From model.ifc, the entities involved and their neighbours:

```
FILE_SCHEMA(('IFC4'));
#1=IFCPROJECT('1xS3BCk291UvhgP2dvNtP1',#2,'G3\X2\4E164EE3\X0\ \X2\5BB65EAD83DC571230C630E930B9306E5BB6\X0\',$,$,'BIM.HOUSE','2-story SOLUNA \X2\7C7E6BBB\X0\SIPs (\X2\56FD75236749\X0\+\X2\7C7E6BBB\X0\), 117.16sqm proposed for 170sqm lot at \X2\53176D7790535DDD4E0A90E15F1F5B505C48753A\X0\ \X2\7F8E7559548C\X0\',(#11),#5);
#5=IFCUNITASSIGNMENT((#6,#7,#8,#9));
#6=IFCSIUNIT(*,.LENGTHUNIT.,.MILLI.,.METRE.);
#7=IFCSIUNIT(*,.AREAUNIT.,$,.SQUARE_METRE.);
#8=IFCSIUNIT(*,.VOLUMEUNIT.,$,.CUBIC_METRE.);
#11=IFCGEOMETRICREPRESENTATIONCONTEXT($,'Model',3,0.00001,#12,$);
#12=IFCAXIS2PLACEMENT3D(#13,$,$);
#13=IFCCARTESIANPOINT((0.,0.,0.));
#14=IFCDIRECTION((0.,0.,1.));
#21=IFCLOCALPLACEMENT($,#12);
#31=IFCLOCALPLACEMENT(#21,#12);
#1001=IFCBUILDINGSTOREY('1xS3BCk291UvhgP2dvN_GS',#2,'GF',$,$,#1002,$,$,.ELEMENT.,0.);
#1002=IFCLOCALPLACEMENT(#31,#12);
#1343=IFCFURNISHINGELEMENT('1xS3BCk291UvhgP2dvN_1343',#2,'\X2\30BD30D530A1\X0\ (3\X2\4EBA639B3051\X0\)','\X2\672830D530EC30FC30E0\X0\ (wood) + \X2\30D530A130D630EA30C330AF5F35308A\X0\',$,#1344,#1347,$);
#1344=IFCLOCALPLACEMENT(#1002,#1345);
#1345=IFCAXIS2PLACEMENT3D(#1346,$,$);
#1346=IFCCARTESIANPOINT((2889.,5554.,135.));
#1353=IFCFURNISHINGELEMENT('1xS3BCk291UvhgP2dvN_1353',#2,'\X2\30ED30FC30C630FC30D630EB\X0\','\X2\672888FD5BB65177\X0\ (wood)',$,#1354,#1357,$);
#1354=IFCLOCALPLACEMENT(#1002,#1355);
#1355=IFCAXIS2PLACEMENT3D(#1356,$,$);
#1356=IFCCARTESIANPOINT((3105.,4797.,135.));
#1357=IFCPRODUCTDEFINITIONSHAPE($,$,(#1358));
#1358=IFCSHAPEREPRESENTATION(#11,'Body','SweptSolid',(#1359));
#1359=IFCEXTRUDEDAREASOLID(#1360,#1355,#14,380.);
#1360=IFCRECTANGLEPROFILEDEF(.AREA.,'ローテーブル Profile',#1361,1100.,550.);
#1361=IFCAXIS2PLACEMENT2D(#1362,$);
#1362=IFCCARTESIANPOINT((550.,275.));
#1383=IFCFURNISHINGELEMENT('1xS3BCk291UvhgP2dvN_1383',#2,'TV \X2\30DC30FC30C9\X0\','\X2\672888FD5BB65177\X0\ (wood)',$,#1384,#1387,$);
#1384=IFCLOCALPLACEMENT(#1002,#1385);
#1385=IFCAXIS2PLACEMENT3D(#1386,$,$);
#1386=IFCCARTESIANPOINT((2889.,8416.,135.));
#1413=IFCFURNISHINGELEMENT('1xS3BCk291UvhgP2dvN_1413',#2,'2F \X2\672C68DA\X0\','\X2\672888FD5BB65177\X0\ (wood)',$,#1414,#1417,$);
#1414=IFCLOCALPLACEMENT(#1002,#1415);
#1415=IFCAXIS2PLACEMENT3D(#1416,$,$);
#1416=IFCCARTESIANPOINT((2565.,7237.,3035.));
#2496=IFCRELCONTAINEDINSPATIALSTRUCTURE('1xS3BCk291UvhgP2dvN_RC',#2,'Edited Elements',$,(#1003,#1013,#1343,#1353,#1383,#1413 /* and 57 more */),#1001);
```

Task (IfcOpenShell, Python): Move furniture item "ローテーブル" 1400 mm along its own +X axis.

```python
import ifcopenshell
import ifcopenshell.api.geometry
import ifcopenshell.util.placement
import ifcopenshell.util.unit

model = ifcopenshell.open("model.ifc")
unit_scale = ifcopenshell.util.unit.calculate_unit_scale(model)

item = model.by_guid("1xS3BCk291UvhgP2dvN_1353")
matrix = ifcopenshell.util.placement.get_local_placement(item.ObjectPlacement)
matrix[:3, 3] += matrix[:3, 0] * 1.4 / unit_scale
ifcopenshell.api.geometry.edit_object_placement(model, product=item, matrix=matrix, is_si=False)

print(ifcopenshell.util.placement.get_local_placement(item.ObjectPlacement).round(3) + 0.0)

model.write("model_updated.ifc")
```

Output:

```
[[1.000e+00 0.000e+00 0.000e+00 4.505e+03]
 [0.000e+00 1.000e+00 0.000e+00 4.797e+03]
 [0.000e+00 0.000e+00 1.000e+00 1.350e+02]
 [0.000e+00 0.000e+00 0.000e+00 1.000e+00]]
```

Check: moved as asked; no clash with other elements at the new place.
